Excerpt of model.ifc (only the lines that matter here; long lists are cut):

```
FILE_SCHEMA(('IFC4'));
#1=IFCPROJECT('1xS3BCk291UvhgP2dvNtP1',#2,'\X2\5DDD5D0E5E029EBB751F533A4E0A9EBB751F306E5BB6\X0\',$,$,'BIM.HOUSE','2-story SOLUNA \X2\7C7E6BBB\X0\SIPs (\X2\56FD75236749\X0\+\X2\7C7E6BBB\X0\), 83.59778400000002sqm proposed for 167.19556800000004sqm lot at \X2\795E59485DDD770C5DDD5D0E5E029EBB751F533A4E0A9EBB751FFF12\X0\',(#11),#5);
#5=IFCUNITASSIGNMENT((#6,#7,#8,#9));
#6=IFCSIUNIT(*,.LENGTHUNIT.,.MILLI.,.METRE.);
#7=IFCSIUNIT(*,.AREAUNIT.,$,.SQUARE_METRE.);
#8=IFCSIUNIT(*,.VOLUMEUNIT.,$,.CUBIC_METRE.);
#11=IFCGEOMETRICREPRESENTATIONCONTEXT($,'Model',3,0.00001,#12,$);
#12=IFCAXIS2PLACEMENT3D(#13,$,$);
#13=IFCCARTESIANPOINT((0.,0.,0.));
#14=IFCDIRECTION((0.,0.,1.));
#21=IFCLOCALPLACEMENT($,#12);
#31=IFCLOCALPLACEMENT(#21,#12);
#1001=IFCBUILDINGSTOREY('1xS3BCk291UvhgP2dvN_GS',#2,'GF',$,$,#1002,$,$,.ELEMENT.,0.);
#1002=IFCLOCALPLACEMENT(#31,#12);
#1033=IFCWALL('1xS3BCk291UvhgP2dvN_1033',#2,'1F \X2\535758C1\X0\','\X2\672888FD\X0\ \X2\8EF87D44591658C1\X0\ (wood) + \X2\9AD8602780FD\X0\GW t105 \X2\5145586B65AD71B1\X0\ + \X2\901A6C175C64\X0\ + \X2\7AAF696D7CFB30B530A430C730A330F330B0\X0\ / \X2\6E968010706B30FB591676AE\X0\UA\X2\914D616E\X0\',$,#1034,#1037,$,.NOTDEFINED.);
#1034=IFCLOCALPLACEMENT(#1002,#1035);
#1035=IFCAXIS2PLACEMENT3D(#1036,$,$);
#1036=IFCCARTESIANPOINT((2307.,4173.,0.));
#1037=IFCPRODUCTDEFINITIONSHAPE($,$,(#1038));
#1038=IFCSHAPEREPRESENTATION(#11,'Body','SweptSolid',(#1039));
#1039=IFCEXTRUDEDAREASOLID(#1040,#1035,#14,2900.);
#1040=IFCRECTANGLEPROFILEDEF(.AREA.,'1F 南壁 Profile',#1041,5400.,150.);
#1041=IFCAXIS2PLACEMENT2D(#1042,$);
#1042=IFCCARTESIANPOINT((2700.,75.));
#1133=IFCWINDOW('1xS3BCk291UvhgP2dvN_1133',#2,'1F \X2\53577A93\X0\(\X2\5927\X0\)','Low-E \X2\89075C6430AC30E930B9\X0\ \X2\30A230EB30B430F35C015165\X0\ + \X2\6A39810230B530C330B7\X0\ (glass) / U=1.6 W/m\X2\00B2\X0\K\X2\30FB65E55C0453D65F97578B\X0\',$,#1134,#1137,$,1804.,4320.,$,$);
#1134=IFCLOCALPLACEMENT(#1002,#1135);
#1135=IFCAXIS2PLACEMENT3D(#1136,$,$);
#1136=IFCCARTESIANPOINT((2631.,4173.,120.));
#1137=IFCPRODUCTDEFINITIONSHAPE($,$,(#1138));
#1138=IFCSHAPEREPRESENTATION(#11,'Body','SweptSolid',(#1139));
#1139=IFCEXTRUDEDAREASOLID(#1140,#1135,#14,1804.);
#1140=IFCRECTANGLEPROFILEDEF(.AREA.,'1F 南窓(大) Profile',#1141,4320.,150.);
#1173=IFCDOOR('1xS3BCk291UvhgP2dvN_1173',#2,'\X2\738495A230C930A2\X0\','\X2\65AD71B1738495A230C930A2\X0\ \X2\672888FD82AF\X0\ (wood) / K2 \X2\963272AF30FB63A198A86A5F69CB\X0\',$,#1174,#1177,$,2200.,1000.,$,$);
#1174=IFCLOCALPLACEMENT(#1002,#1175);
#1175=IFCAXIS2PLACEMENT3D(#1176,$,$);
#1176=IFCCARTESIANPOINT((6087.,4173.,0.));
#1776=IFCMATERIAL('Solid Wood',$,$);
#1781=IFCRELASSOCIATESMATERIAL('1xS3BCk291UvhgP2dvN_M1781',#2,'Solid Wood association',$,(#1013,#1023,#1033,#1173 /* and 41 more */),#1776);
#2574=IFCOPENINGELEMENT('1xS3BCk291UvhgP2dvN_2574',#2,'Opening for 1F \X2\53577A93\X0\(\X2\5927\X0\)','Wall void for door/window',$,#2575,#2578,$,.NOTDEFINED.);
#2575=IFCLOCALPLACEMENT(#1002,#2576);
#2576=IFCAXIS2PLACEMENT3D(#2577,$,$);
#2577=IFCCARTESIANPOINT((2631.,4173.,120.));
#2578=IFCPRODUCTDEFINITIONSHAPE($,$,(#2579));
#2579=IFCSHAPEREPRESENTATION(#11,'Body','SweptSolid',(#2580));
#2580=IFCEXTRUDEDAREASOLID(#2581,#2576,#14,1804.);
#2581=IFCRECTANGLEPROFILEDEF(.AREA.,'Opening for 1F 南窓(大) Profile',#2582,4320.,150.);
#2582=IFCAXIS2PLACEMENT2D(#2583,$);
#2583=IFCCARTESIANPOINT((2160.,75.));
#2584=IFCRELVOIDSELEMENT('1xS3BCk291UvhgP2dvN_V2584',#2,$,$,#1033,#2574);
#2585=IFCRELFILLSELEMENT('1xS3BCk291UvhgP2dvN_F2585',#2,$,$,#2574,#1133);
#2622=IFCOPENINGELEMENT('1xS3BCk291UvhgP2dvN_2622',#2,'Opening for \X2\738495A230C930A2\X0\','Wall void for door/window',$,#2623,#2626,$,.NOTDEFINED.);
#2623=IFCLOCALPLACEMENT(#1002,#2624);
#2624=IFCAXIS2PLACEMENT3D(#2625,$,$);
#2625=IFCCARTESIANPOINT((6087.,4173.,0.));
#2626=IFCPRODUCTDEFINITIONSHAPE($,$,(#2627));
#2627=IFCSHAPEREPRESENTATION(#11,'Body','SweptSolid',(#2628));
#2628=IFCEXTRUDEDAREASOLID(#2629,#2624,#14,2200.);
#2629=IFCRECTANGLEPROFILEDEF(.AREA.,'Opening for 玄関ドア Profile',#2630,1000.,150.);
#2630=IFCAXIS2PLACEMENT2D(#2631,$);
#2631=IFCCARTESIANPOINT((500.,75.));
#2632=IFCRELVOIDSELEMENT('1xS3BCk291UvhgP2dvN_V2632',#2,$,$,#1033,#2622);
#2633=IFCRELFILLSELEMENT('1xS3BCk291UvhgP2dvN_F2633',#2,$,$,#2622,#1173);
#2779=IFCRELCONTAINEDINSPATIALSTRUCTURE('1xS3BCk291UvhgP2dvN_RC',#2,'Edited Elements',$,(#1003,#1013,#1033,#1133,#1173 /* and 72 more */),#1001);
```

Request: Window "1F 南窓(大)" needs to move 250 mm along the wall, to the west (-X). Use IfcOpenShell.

```python
import ifcopenshell
import ifcopenshell.api.geometry
import ifcopenshell.util.placement
import ifcopenshell.util.unit

model = ifcopenshell.open("model.ifc")
unit_scale = ifcopenshell.util.unit.calculate_unit_scale(model)

window = model.by_id(1133)
opening = window.FillsVoids[0].RelatingOpeningElement
wall = opening.VoidsElements[0].RelatingBuildingElement

wall_matrix = ifcopenshell.util.placement.get_local_placement(wall.ObjectPlacement)
shift = wall_matrix[:3, 0] * -0.25 / unit_scale
before = ifcopenshell.util.placement.get_local_placement(window.ObjectPlacement)[:3, 3].copy()

# The window is not placed relative to its opening, so move both.
for product in (opening, window):
    matrix = ifcopenshell.util.placement.get_local_placement(product.ObjectPlacement)
    matrix[:3, 3] += shift
    ifcopenshell.api.geometry.edit_object_placement(model, product=product, matrix=matrix, is_si=False)

after = ifcopenshell.util.placement.get_local_placement(window.ObjectPlacement)[:3, 3]
print("window moved by", (after - before).round(3) + 0.0)

model.write("model_updated.ifc")
```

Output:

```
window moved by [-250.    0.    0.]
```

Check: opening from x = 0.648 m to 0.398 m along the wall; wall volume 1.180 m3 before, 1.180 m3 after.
